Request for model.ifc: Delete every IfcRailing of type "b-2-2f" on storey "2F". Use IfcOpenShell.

First a look at what the model holds.

```python
import ifcopenshell
import ifcopenshell.util.element

model = ifcopenshell.open("model.ifc")
print(model.schema)
storey = next(s for s in model.by_type("IfcBuildingStorey") if s.Name == "2F")
railings = [e for e in ifcopenshell.util.element.get_decomposition(storey) if e.is_a("IfcRailing")]
seen = {}
for e in railings:
    element_type = ifcopenshell.util.element.get_type(e)
    name = element_type.Name if element_type not in (None, e) else None
    seen[name] = seen.get(name, 0) + 1
for name, count in sorted(seen.items(), key=str):
    print(count, "x", name)
```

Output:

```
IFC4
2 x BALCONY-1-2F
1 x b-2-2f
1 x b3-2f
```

```python
import ifcopenshell
import ifcopenshell.api.root
import ifcopenshell.util.element

model = ifcopenshell.open("model.ifc")

storey = next(s for s in model.by_type("IfcBuildingStorey") if s.Name == "2F")
railings = [e for e in ifcopenshell.util.element.get_decomposition(storey) if e.is_a("IfcRailing")]
targets = [e for e in railings if (t := ifcopenshell.util.element.get_type(e)) not in (None, e) and t.Name == "b-2-2f"]

for e in targets:
    ifcopenshell.api.root.remove_product(model, product=e)
print(len(targets), "removed")

model.write("model-out.ifc")
```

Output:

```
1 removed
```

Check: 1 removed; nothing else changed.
